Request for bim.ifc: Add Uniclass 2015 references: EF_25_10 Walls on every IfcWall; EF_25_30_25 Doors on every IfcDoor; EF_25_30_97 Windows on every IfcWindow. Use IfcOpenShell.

First a look at what the model holds.

```python
import ifcopenshell

model = ifcopenshell.open("bim.ifc")
print(model.schema)
print("classifications:", [c.Name for c in model.by_type("IfcClassification")])
for ifc_class in ("IfcDoor", "IfcRoof", "IfcStair", "IfcWall", "IfcWindow"):
    print(ifc_class, len(model.by_type(ifc_class)))
```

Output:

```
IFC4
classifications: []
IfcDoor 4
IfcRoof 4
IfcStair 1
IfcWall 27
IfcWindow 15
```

```python
import ifcopenshell
import ifcopenshell.api.classification

model = ifcopenshell.open("bim.ifc")

system = ifcopenshell.api.classification.add_classification(model, classification="Uniclass 2015")

codes = {
    "IfcWall": ("EF_25_10", "Walls"),
    "IfcDoor": ("EF_25_30_25", "Doors"),
    "IfcWindow": ("EF_25_30_97", "Windows"),
}
for ifc_class, (code, name) in codes.items():
    products = model.by_type(ifc_class)
    ifcopenshell.api.classification.add_reference(
        model, products=products, classification=system, identification=code, name=name
    )
    print(code, len(products))

model.write("bim_updated.ifc")
```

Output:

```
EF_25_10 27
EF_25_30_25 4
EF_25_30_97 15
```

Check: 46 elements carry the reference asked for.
